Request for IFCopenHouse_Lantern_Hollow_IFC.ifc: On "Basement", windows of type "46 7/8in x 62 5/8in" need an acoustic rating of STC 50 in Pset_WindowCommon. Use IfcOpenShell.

First a look at what the model holds.

```python
import ifcopenshell
import ifcopenshell.util.element

model = ifcopenshell.open("IFCopenHouse_Lantern_Hollow_IFC.ifc")
print(model.schema)
storey = next(s for s in model.by_type("IfcBuildingStorey") if s.Name == "Basement")
windows = [e for e in ifcopenshell.util.element.get_decomposition(storey) if e.is_a("IfcWindow")]
seen = {}
for e in windows:
    element_type = ifcopenshell.util.element.get_type(e)
    key = (element_type.Name if element_type != e and element_type else None, ifcopenshell.util.element.get_pset(e, "Pset_WindowCommon", "AcousticRating"))
    seen[key] = seen.get(key, 0) + 1
for (name, value), count in sorted(seen.items(), key=str):
    print(count, "x", name, "|", value)
```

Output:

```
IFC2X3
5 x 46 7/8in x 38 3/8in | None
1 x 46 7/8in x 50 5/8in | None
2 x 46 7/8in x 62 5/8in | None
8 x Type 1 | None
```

```python
import ifcopenshell
import ifcopenshell.api.pset
import ifcopenshell.util.element

model = ifcopenshell.open("IFCopenHouse_Lantern_Hollow_IFC.ifc")

storey = next(s for s in model.by_type("IfcBuildingStorey") if s.Name == "Basement")
windows = [e for e in ifcopenshell.util.element.get_decomposition(storey) if e.is_a("IfcWindow")]

count = 0
for e in windows:
    element_type = ifcopenshell.util.element.get_type(e)
    if element_type in (None, e) or element_type.Name != "46 7/8in x 62 5/8in":
        continue
    # add_pset returns the element's existing set when there is one.
    pset = ifcopenshell.api.pset.add_pset(model, product=e, name="Pset_WindowCommon")
    ifcopenshell.api.pset.edit_pset(model, pset=pset, properties={"AcousticRating": "STC 50"})
    count += 1

print(count, "windows updated")

model.write("IFCopenHouse_Lantern_Hollow_IFC-out.ifc")
```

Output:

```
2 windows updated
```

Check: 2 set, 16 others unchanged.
